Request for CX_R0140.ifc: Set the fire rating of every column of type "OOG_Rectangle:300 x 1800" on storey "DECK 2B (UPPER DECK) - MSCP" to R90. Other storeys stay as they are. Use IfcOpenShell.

First a look at what the model holds.

```python
import ifcopenshell
import ifcopenshell.util.element

model = ifcopenshell.open("CX_R0140.ifc")
print(model.schema)
storey = next(s for s in model.by_type("IfcBuildingStorey") if s.Name == "DECK 2B (UPPER DECK) - MSCP")
columns = [e for e in ifcopenshell.util.element.get_decomposition(storey) if e.is_a("IfcColumn")]
seen = {}
for e in columns:
    element_type = ifcopenshell.util.element.get_type(e)
    key = (element_type.Name if element_type != e and element_type else None, ifcopenshell.util.element.get_pset(e, "Pset_ColumnCommon", "FireRating"))
    seen[key] = seen.get(key, 0) + 1
for (name, value), count in sorted(seen.items(), key=str):
    print(count, "x", name, "|", value)
```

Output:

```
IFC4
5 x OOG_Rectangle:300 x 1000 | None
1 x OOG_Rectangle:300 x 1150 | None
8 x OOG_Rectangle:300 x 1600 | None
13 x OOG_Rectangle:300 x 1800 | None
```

```python
import ifcopenshell
import ifcopenshell.api.pset
import ifcopenshell.util.element

model = ifcopenshell.open("CX_R0140.ifc")

storey = next(s for s in model.by_type("IfcBuildingStorey") if s.Name == "DECK 2B (UPPER DECK) - MSCP")
columns = [e for e in ifcopenshell.util.element.get_decomposition(storey) if e.is_a("IfcColumn")]

count = 0
for e in columns:
    element_type = ifcopenshell.util.element.get_type(e)
    if element_type in (None, e) or element_type.Name != "OOG_Rectangle:300 x 1800":
        continue
    # add_pset returns the element's existing set when there is one.
    pset = ifcopenshell.api.pset.add_pset(model, product=e, name="Pset_ColumnCommon")
    ifcopenshell.api.pset.edit_pset(model, pset=pset, properties={"FireRating": "R90"})
    count += 1

print(count, "columns updated")

model.write("CX_R0140_rev.ifc")
```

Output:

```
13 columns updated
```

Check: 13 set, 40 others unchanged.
